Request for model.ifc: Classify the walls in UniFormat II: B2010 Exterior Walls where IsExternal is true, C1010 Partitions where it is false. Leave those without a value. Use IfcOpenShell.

First a look at what the model holds.

```python
import ifcopenshell
import ifcopenshell.util.element

model = ifcopenshell.open("model.ifc")
print(model.schema)
print("classifications:", [c.Name for c in model.by_type("IfcClassification")])
values = [ifcopenshell.util.element.get_pset(e, "Pset_WallCommon", "IsExternal") for e in model.by_type("IfcWall")]
for value in (True, False, None):
    print("IsExternal", value, values.count(value))
```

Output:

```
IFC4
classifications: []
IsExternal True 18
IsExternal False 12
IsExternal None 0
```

```python
import ifcopenshell
import ifcopenshell.api.classification
import ifcopenshell.util.element

model = ifcopenshell.open("model.ifc")

system = ifcopenshell.api.classification.add_classification(model, classification="UniFormat II")

walls = model.by_type("IfcWall")
external = {e: ifcopenshell.util.element.get_pset(e, "Pset_WallCommon", "IsExternal") for e in walls}
for flag, code, name in ((True, "B2010", "Exterior Walls"), (False, "C1010", "Partitions")):
    products = [e for e in walls if external[e] is flag]
    ifcopenshell.api.classification.add_reference(
        model, products=products, classification=system, identification=code, name=name
    )
    print(code, len(products))

model.write("model_rev.ifc")
```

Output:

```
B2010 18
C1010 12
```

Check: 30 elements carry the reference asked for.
